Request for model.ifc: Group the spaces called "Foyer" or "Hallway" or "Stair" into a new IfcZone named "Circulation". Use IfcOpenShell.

First a look at what the model holds.

```python
import ifcopenshell

model = ifcopenshell.open("model.ifc")
print(model.schema)
seen = {}
for space in model.by_type("IfcSpace"):
    seen[space.LongName] = seen.get(space.LongName, 0) + 1
for name, count in sorted(seen.items(), key=str):
    print(count, "x", name)
print("zones:", [z.Name for z in model.by_type("IfcZone")][:20])
```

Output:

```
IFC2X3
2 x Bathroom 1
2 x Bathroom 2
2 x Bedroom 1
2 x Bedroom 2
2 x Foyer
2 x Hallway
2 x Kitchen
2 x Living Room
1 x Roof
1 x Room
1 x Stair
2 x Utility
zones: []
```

```python
import ifcopenshell
import ifcopenshell.api.group
import ifcopenshell.api.root

model = ifcopenshell.open("model.ifc")

names = {"Foyer", "Hallway", "Stair"}
spaces = [s for s in model.by_type("IfcSpace") if s.LongName in names]

zone = ifcopenshell.api.root.create_entity(model, ifc_class="IfcZone", name="Circulation")
ifcopenshell.api.group.assign_group(model, products=spaces, group=zone)
print(len(spaces), "spaces in", zone.Name)

model.write("model_v2.ifc")
```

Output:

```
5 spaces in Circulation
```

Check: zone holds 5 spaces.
